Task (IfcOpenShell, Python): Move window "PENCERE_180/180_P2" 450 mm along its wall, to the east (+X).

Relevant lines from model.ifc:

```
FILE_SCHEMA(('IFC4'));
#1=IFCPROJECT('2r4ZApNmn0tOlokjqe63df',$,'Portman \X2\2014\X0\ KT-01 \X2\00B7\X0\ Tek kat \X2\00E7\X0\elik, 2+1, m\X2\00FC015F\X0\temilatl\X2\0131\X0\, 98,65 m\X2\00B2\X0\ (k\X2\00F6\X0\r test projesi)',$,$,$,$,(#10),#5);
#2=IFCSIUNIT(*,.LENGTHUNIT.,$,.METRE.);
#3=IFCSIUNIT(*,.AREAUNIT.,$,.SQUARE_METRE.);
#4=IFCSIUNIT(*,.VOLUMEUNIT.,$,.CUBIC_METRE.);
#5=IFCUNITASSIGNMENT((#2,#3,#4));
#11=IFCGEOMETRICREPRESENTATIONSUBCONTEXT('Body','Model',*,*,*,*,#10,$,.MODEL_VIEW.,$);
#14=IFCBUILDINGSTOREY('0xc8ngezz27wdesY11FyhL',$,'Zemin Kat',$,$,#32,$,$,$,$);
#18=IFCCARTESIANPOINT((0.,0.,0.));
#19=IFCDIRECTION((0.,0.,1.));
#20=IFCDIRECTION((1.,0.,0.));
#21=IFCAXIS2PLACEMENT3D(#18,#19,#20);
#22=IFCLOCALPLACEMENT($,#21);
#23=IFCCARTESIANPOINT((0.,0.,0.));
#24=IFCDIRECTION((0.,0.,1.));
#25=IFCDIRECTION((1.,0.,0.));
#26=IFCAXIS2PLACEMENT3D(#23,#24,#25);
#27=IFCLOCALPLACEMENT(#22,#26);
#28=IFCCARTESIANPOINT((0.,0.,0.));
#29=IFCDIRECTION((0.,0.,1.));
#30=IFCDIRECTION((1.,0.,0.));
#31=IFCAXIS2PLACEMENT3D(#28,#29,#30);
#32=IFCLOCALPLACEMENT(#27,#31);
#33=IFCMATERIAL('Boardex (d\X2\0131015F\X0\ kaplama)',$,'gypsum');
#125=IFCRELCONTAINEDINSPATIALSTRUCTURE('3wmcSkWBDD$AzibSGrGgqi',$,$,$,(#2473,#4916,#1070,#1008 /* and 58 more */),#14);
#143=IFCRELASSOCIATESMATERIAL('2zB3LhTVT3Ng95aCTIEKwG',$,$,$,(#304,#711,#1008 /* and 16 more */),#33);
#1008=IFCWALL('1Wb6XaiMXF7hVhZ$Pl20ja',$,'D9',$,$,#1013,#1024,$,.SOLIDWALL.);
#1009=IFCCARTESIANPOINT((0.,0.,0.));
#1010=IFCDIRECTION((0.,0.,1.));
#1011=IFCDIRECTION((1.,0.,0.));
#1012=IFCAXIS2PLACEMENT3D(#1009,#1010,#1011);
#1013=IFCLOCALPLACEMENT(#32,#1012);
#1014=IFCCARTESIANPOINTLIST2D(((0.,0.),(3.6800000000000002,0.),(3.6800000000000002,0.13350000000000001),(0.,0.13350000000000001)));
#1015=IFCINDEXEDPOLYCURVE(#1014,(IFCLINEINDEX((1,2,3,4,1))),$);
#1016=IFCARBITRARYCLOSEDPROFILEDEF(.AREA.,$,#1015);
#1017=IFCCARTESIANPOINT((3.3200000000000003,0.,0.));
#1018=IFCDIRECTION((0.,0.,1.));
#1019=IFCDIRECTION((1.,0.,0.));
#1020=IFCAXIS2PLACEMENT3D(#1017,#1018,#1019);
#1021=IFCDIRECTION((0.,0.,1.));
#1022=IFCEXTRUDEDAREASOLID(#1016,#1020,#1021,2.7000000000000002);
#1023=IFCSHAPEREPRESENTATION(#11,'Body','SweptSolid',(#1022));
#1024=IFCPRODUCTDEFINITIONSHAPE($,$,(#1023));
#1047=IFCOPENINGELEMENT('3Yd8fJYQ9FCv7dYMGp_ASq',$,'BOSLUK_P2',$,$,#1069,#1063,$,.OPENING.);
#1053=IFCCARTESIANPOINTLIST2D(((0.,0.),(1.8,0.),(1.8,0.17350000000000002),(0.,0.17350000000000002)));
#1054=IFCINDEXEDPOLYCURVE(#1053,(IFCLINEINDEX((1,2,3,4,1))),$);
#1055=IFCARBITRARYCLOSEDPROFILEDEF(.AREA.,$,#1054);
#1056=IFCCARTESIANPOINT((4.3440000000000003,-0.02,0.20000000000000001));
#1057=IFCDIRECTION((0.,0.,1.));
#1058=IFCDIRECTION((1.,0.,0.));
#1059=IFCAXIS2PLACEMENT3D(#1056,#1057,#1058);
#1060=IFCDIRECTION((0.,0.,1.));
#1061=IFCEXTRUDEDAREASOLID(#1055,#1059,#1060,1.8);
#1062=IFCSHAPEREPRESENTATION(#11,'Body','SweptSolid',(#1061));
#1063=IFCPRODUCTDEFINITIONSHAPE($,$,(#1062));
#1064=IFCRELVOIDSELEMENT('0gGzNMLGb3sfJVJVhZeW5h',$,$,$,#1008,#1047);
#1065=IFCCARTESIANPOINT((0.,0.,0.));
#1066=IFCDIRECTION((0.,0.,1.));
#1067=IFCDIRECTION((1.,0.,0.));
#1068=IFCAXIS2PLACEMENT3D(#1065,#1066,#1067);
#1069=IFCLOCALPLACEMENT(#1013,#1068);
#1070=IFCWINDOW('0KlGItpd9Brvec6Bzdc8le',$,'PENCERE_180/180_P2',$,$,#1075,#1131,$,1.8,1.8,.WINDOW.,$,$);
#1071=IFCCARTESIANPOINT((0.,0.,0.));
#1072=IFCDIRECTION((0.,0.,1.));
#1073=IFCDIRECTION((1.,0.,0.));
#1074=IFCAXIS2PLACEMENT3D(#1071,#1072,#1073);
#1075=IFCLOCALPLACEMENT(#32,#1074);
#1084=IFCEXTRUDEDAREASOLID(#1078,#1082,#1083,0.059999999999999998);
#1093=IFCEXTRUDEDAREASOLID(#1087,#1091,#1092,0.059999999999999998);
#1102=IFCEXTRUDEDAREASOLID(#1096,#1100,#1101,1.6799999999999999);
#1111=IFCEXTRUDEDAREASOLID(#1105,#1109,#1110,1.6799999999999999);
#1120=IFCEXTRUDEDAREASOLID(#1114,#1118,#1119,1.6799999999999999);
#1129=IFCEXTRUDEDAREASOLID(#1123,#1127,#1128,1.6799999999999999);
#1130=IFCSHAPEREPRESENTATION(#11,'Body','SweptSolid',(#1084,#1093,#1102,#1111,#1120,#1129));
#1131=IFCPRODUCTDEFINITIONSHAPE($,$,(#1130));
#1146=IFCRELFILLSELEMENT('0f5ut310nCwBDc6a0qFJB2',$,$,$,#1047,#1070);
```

```python
import ifcopenshell
import ifcopenshell.api.geometry
import ifcopenshell.util.placement

model = ifcopenshell.open("model.ifc")

window = model.by_id(1070)
opening = window.FillsVoids[0].RelatingOpeningElement
wall = opening.VoidsElements[0].RelatingBuildingElement

wall_matrix = ifcopenshell.util.placement.get_local_placement(wall.ObjectPlacement)
shift = wall_matrix[:3, 0] * 0.45
before = ifcopenshell.util.placement.get_local_placement(window.ObjectPlacement)[:3, 3].copy()

# The window is not placed relative to its opening, so move both.
for product in (opening, window):
    matrix = ifcopenshell.util.placement.get_local_placement(product.ObjectPlacement)
    matrix[:3, 3] += shift
    ifcopenshell.api.geometry.edit_object_placement(model, product=product, matrix=matrix, is_si=False)

after = ifcopenshell.util.placement.get_local_placement(window.ObjectPlacement)[:3, 3]
print("window moved by", (after - before).round(3) + 0.0)

model.write("model_edited.ifc")
```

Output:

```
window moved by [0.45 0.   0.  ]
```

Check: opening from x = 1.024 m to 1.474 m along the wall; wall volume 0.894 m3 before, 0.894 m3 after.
